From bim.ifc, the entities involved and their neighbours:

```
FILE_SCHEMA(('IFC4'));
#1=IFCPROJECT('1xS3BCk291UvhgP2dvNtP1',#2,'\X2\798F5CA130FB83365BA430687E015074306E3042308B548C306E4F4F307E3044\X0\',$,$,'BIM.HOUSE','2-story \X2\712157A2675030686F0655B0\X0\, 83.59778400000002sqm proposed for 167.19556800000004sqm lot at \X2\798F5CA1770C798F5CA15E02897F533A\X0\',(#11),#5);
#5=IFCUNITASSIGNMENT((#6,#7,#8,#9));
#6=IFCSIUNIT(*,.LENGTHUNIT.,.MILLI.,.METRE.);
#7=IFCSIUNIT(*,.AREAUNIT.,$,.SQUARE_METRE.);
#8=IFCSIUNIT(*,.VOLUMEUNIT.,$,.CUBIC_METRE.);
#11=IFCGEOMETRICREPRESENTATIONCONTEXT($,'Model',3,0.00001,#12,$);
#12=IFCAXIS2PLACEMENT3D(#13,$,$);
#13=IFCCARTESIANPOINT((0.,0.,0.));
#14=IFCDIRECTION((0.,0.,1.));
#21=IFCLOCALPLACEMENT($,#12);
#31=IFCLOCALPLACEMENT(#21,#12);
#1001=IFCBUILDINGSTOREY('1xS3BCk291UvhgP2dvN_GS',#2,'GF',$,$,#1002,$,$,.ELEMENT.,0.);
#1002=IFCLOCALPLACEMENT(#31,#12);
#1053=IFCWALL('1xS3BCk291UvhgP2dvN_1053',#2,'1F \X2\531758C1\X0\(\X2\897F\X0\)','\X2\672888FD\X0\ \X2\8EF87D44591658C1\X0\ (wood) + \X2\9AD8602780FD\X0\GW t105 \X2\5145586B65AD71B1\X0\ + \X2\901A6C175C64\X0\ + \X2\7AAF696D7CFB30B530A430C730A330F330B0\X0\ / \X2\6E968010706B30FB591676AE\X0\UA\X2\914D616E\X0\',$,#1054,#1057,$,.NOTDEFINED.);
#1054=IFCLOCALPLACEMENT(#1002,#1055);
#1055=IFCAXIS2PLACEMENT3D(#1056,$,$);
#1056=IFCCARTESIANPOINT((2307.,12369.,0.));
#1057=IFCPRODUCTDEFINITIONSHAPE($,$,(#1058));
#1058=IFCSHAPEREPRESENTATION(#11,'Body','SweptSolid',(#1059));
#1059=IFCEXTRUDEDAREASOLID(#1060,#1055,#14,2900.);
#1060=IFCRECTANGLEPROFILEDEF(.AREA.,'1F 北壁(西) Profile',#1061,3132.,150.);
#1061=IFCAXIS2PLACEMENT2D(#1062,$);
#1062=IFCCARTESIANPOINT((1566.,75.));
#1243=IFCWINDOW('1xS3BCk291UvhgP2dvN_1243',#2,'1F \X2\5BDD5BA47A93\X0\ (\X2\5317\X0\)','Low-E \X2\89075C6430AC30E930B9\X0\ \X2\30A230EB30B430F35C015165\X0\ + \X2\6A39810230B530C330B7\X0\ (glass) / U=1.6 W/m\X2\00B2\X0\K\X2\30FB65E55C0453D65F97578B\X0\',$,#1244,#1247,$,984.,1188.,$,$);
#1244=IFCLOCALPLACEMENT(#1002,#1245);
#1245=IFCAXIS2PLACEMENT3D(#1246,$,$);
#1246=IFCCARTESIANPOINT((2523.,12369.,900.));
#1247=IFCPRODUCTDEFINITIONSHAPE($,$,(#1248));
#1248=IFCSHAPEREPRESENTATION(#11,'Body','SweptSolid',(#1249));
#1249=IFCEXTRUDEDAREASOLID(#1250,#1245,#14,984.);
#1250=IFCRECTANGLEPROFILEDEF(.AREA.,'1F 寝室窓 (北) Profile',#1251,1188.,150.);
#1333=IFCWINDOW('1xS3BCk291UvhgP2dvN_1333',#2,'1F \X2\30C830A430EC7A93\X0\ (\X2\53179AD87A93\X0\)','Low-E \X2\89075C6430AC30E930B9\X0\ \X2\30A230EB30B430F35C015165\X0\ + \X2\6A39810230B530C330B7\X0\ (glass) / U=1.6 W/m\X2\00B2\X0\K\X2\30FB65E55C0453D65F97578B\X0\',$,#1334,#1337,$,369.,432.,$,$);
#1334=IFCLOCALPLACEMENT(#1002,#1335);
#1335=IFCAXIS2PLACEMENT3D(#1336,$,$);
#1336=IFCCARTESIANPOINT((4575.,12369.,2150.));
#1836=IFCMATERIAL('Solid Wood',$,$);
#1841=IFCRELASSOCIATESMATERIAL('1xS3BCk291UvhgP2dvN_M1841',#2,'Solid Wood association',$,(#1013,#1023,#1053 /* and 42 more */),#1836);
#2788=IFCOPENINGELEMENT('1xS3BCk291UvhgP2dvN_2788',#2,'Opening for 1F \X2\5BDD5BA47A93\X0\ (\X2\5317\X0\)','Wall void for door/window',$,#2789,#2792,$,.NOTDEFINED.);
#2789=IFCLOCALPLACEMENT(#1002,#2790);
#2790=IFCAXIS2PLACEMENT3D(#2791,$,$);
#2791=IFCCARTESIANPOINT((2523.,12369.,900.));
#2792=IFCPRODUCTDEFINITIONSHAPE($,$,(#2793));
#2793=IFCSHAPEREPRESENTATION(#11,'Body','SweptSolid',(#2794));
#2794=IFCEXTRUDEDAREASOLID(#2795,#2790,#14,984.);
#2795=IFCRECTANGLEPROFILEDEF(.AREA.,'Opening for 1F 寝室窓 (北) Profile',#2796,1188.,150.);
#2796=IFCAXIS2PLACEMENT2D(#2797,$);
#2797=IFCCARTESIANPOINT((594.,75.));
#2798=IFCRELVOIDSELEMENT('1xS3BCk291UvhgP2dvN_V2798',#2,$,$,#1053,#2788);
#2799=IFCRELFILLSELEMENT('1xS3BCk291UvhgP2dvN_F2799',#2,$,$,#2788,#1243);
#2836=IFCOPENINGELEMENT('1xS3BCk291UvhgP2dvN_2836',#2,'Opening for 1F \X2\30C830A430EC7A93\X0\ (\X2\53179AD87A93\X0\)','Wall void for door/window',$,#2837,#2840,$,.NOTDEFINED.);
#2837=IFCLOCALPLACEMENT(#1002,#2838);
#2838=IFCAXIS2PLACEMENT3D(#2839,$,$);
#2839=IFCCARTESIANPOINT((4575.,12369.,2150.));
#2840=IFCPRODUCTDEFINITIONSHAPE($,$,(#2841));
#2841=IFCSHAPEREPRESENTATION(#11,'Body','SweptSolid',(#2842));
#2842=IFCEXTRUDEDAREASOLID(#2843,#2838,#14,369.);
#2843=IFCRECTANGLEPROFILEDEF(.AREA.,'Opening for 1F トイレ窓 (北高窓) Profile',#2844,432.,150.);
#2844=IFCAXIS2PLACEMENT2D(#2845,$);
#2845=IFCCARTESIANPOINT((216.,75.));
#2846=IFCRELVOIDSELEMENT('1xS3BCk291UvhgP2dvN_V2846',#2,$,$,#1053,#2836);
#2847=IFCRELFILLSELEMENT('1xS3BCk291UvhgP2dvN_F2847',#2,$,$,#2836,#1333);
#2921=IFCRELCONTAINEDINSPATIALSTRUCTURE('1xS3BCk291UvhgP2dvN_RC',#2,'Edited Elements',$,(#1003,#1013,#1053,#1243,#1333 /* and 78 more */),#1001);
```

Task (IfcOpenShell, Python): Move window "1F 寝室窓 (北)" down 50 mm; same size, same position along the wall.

```python
import numpy as np
import ifcopenshell
import ifcopenshell.api.geometry
import ifcopenshell.util.placement
import ifcopenshell.util.unit

model = ifcopenshell.open("bim.ifc")
unit_scale = ifcopenshell.util.unit.calculate_unit_scale(model)

window = model.by_guid("1xS3BCk291UvhgP2dvN_1243")
opening = window.FillsVoids[0].RelatingOpeningElement
dz = -50.0

shift = np.array([0.0, 0.0, dz])
# The window is not placed relative to its opening, so move both.
for product in (opening, window):
    matrix = ifcopenshell.util.placement.get_local_placement(product.ObjectPlacement)
    matrix[:3, 3] += shift
    ifcopenshell.api.geometry.edit_object_placement(model, product=product, matrix=matrix, is_si=False)

print(f"moved by {dz * unit_scale:+.3f} m")

model.write("bim_edited.ifc")
```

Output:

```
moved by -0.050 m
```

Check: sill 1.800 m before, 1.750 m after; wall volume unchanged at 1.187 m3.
